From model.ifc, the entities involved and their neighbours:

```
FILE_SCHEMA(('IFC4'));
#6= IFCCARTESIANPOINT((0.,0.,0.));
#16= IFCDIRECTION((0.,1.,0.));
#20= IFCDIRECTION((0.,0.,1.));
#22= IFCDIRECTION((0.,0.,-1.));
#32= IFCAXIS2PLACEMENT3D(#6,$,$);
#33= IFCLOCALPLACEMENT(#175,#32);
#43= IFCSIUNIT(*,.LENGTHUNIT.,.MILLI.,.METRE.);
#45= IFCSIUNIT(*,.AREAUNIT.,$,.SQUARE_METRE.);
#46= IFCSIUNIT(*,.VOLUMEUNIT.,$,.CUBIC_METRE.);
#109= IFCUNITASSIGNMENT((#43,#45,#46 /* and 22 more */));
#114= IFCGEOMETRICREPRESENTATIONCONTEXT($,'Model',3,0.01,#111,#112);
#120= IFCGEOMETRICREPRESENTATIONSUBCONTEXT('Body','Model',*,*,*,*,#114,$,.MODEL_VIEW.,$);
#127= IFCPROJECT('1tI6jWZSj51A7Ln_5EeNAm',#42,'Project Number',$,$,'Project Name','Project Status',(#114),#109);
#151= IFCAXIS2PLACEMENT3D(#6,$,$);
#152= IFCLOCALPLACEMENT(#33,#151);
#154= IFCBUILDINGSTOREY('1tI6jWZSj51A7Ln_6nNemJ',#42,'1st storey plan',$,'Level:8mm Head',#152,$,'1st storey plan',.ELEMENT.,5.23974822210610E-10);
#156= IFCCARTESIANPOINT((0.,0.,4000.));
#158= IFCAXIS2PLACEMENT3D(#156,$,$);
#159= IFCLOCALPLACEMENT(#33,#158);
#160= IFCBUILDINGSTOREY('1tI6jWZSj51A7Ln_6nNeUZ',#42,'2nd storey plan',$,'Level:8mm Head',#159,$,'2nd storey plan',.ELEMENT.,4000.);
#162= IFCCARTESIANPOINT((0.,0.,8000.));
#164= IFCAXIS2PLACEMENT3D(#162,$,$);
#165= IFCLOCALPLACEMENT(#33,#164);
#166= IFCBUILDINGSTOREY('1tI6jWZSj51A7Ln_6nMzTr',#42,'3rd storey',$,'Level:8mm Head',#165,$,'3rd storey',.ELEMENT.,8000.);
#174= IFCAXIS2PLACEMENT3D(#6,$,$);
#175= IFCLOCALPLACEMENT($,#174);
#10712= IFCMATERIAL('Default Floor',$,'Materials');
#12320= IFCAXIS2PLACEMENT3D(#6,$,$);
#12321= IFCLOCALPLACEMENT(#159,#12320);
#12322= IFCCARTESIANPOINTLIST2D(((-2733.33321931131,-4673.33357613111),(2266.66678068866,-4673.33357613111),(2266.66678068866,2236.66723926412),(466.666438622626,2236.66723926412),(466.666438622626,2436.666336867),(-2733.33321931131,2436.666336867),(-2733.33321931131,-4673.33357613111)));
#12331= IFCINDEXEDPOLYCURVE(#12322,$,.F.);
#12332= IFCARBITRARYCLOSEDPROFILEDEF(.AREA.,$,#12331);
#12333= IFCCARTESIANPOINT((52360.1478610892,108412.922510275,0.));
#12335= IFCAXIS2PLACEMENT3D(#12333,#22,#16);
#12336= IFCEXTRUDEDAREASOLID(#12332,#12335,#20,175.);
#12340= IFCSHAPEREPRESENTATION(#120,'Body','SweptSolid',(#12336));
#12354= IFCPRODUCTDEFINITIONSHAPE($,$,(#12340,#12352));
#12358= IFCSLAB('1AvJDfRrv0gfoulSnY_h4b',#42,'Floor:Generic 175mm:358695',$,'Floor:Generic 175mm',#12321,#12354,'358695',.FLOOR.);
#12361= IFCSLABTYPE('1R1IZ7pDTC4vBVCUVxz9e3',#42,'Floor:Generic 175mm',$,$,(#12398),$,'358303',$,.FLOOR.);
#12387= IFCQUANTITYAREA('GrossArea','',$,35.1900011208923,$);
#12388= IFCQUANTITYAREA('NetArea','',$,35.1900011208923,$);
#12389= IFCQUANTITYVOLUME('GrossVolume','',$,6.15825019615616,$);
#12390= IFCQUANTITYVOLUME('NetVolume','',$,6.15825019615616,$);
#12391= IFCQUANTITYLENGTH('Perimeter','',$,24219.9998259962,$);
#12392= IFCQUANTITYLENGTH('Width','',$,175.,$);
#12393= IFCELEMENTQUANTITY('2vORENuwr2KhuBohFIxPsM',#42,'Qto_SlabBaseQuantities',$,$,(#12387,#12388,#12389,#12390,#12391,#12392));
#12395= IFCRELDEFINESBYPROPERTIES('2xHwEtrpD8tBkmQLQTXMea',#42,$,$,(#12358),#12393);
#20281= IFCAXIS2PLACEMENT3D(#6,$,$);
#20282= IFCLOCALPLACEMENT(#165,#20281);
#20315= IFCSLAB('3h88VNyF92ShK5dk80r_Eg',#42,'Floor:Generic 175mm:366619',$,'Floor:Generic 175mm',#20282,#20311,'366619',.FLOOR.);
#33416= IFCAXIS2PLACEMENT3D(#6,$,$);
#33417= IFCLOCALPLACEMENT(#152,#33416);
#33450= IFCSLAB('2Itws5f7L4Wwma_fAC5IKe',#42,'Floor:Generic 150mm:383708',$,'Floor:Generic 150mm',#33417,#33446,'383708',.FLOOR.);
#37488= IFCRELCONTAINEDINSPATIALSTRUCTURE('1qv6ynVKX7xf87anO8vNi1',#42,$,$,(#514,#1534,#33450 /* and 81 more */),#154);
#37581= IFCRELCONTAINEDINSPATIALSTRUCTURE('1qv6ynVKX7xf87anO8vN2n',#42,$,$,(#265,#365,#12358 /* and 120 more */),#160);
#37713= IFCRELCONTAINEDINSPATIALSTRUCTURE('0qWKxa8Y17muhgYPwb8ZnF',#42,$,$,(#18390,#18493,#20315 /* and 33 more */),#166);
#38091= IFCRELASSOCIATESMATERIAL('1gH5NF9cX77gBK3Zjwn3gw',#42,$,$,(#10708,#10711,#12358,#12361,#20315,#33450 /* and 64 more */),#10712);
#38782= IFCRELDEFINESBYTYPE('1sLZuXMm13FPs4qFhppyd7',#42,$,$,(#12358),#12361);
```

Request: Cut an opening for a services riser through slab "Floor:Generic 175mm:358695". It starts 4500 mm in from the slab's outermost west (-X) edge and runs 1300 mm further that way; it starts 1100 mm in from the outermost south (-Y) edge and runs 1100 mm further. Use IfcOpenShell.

```python
import numpy as np
import ifcopenshell
import ifcopenshell.api.feature
import ifcopenshell.api.geometry
import ifcopenshell.api.pset
import ifcopenshell.api.root
import ifcopenshell.geom
import ifcopenshell.util.element
import ifcopenshell.util.placement
import ifcopenshell.util.representation
import ifcopenshell.util.shape
import ifcopenshell.util.unit

model = ifcopenshell.open("model.ifc")
unit_scale = ifcopenshell.util.unit.calculate_unit_scale(model)
area_scale = ifcopenshell.util.unit.calculate_unit_scale(model, "AREAUNIT")
volume_scale = ifcopenshell.util.unit.calculate_unit_scale(model, "VOLUMEUNIT")
settings = ifcopenshell.geom.settings()


def volume(element):
    """Net volume in cubic metres, openings subtracted."""
    shape = ifcopenshell.geom.create_shape(settings, element)
    return ifcopenshell.util.shape.get_volume(shape.geometry)


slab = model.by_guid("1AvJDfRrv0gfoulSnY_h4b")
before = volume(slab)

# Extent in the slab's own axes, in metres. The edges named are its -X and -Y sides.
slab_shape = ifcopenshell.geom.create_shape(settings, slab)
vertices = ifcopenshell.util.shape.get_vertices(slab_shape.geometry)
x_min, y_min, bottom = vertices.min(axis=0)
top = vertices[:, 2].max()

opening = ifcopenshell.api.root.create_entity(model, ifc_class="IfcOpeningElement", name="Services riser opening", predefined_type="OPENING")
context = ifcopenshell.util.representation.get_context(model, "Model", "Body", "MODEL_VIEW")
width, depth = 1.3, 1.1
outline = [(0.0, 0.0), (width, 0.0), (width, depth), (0.0, depth), (0.0, 0.0)]
# Overshoot both faces by 50 mm so the cut is clean.
shape = ifcopenshell.api.geometry.add_slab_representation(
    model, context=context, depth=top - bottom + 0.1, polyline=outline
)
ifcopenshell.api.geometry.assign_representation(model, product=opening, representation=shape)

matrix = ifcopenshell.util.placement.get_local_placement(slab.ObjectPlacement)
matrix[:, 3] = matrix @ np.append(np.array([x_min + 4.5, y_min + 1.1, bottom - 0.05]) / unit_scale, 1.0)
ifcopenshell.api.geometry.edit_object_placement(model, product=opening, matrix=matrix, is_si=False)
ifcopenshell.api.feature.add_feature(model, feature=opening, element=slab)

after = volume(slab)

# Update the slab's stored quantities.
qto = model.by_id(ifcopenshell.util.element.get_pset(slab, "Qto_SlabBaseQuantities", should_inherit=False)["id"])
ifcopenshell.api.pset.edit_qto(model, qto=qto, properties={
    "NetArea": after / (top - bottom) / area_scale,
    "NetVolume": after / volume_scale,
})

print(f"slab volume {before:.3f} -> {after:.3f} m3")

model.write("model_rev.ifc")
```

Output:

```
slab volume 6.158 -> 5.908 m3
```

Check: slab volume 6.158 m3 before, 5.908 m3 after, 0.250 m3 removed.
